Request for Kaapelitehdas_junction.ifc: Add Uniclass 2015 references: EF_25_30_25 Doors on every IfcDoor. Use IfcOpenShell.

First a look at what the model holds.

```python
import ifcopenshell

model = ifcopenshell.open("Kaapelitehdas_junction.ifc")
print(model.schema)
print("classifications:", [c.Name for c in model.by_type("IfcClassification")])
for ifc_class in ("IfcDoor", "IfcRoof", "IfcStair", "IfcWall", "IfcWindow"):
    print(ifc_class, len(model.by_type(ifc_class)))
```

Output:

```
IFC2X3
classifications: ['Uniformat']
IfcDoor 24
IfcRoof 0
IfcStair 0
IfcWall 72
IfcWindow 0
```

```python
import ifcopenshell
import ifcopenshell.api.classification

model = ifcopenshell.open("Kaapelitehdas_junction.ifc")

# IFC2X3 requires Source and Edition and has no link from the project to the system.
system = model.create_entity("IfcClassification", Source="NBS", Edition="2015", Name="Uniclass 2015")

codes = {
    "IfcDoor": ("EF_25_30_25", "Doors"),
}
for ifc_class, (code, name) in codes.items():
    products = model.by_type(ifc_class)
    ifcopenshell.api.classification.add_reference(
        model, products=products, classification=system, identification=code, name=name
    )
    print(code, len(products))

model.write("Kaapelitehdas_junction_v2.ifc")
```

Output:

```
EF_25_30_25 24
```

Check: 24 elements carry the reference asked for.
